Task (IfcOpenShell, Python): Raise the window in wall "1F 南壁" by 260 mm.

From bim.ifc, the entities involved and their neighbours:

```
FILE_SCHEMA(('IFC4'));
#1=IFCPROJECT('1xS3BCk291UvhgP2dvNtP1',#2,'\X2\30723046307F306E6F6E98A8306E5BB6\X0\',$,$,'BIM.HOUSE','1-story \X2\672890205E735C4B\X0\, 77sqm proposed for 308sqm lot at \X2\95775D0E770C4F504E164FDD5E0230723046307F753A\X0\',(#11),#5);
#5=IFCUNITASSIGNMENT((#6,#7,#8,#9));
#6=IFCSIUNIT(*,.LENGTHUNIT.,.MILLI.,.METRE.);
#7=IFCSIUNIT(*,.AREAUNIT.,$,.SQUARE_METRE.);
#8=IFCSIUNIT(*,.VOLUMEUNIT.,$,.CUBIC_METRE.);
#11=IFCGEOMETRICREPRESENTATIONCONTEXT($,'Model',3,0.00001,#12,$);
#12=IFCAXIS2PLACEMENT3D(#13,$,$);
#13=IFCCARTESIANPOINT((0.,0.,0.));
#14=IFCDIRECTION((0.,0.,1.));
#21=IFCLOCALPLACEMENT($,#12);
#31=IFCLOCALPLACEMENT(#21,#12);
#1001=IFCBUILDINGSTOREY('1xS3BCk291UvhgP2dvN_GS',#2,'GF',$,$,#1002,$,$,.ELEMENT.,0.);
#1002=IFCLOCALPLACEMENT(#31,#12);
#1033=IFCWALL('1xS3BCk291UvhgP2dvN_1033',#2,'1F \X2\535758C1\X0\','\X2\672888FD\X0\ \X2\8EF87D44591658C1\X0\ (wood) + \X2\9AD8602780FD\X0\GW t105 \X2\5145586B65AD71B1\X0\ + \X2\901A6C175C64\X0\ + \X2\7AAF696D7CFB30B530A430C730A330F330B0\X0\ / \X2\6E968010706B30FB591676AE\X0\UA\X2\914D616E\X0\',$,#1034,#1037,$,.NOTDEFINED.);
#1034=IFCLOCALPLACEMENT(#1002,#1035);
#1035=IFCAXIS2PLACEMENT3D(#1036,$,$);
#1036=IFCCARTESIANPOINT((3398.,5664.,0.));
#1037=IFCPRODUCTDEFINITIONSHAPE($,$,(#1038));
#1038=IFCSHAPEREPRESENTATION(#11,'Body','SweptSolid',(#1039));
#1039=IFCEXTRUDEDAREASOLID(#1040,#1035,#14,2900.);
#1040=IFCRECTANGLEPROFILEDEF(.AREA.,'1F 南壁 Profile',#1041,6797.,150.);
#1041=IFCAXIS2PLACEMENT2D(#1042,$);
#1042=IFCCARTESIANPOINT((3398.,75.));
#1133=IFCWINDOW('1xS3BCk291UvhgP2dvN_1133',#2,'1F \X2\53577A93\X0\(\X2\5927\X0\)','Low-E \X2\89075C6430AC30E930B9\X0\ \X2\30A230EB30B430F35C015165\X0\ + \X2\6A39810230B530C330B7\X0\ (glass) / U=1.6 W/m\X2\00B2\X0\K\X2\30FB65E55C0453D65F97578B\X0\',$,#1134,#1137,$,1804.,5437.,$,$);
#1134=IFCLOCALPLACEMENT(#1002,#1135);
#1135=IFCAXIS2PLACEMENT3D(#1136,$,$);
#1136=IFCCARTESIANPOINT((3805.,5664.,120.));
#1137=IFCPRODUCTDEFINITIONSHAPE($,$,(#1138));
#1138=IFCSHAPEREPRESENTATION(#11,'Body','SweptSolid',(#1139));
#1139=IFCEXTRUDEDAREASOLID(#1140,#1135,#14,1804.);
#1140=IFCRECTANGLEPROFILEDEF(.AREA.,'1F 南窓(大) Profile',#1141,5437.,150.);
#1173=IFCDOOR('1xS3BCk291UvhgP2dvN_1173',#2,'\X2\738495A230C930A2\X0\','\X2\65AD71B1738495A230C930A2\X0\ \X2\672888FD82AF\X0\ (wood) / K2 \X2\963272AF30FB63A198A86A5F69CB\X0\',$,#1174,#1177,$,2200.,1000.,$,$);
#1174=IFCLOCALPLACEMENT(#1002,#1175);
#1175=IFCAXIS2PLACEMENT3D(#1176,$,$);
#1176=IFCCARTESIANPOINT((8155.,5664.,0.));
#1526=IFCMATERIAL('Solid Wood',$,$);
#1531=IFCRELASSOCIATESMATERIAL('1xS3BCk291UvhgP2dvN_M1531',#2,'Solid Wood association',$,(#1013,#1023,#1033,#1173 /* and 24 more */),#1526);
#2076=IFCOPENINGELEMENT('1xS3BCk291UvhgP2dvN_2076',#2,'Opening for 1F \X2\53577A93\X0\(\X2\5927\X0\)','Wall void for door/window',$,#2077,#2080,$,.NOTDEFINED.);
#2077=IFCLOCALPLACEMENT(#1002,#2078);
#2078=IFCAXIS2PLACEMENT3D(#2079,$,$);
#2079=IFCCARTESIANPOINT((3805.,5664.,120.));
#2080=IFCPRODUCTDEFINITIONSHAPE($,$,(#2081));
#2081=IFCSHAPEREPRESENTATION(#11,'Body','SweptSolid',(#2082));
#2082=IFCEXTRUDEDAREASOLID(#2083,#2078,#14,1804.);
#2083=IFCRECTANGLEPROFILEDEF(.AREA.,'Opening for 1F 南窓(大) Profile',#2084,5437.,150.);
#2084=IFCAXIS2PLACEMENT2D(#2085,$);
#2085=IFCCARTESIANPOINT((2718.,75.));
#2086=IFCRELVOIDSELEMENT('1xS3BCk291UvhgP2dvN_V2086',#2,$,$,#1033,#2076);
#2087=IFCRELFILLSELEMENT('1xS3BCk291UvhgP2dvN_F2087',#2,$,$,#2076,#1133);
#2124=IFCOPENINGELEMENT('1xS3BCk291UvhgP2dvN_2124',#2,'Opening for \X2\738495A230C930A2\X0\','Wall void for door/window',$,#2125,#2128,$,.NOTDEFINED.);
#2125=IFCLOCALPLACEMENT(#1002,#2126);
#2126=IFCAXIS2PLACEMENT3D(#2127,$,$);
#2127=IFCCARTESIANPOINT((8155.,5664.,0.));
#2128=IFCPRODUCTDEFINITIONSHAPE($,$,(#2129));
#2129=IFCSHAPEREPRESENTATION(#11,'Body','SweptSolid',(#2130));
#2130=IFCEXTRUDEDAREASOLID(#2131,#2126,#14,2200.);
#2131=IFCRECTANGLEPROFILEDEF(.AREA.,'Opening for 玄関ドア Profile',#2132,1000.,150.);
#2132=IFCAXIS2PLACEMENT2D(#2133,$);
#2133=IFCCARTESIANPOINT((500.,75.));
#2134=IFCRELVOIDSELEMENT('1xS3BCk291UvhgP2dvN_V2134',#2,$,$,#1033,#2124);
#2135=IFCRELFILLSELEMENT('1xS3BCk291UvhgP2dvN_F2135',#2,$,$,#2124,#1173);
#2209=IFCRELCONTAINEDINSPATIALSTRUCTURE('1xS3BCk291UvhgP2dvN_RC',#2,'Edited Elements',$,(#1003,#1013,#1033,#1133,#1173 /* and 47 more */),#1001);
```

```python
import numpy as np
import ifcopenshell
import ifcopenshell.api.geometry
import ifcopenshell.util.placement
import ifcopenshell.util.unit

model = ifcopenshell.open("bim.ifc")
unit_scale = ifcopenshell.util.unit.calculate_unit_scale(model)

window = model.by_guid("1xS3BCk291UvhgP2dvN_1133")
opening = window.FillsVoids[0].RelatingOpeningElement
dz = 0.26 / unit_scale

shift = np.array([0.0, 0.0, dz])
# The window is not placed relative to its opening, so move both.
for product in (opening, window):
    matrix = ifcopenshell.util.placement.get_local_placement(product.ObjectPlacement)
    matrix[:3, 3] += shift
    ifcopenshell.api.geometry.edit_object_placement(model, product=product, matrix=matrix, is_si=False)

print(f"moved by {dz * unit_scale:+.3f} m")

model.write("bim_rev.ifc")
```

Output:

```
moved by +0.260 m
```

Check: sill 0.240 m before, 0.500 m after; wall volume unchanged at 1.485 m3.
